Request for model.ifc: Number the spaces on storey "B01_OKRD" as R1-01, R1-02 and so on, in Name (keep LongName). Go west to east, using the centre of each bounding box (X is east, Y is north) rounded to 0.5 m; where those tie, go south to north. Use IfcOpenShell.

First a look at what the model holds.

```python
import ifcopenshell
import ifcopenshell.util.element
import ifcopenshell.util.placement

model = ifcopenshell.open("model.ifc")
print(model.schema)
storey = next(s for s in model.by_type("IfcBuildingStorey") if s.Name == "B01_OKRD")
spaces = [e for e in ifcopenshell.util.element.get_decomposition(storey) if e.is_a("IfcSpace")]
for e in sorted(spaces, key=lambda e: e.id()):
    origin = ifcopenshell.util.placement.get_local_placement(e.ObjectPlacement)[:3, 3]
    print(e.id(), e.Name, e.LongName, origin.round(2) + 0.0, sep=" | ")
```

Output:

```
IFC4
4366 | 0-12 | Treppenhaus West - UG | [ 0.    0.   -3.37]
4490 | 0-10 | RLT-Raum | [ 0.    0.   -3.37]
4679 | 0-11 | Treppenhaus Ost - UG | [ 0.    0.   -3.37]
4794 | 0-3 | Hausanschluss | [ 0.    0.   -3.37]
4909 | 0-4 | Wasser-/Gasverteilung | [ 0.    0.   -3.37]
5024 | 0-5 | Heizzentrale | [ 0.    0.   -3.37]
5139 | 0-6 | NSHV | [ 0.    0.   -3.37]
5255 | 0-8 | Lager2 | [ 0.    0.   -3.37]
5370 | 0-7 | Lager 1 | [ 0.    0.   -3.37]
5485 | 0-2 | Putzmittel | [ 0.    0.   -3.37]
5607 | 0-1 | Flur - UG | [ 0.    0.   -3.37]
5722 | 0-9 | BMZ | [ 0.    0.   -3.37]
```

```python
import ifcopenshell
import ifcopenshell.geom
import ifcopenshell.util.element
import ifcopenshell.util.shape

model = ifcopenshell.open("model.ifc")
settings = ifcopenshell.geom.settings()
settings.set("use-world-coords", True)


def centre(element):
    shape = ifcopenshell.geom.create_shape(settings, element)
    return ifcopenshell.util.shape.get_bbox_centroid(shape.geometry)


storey = next(s for s in model.by_type("IfcBuildingStorey") if s.Name == "B01_OKRD")
spaces = [e for e in ifcopenshell.util.element.get_decomposition(storey) if e.is_a("IfcSpace")]

# Insertion points can sit at a corner or the storey origin, so sort by the geometry (in metres).
centres = {e: centre(e) for e in spaces}
spaces.sort(key=lambda e: (round(centres[e][0] / 0.5), centres[e][1]))

for i, e in enumerate(spaces, start=1):
    number = f"R1-{i:02d}"
    e.Name = number
    print(e.id(), number)

model.write("model_v2.ifc")
```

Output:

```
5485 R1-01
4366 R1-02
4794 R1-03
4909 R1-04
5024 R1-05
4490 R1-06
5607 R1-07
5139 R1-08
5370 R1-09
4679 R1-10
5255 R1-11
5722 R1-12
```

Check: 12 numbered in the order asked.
